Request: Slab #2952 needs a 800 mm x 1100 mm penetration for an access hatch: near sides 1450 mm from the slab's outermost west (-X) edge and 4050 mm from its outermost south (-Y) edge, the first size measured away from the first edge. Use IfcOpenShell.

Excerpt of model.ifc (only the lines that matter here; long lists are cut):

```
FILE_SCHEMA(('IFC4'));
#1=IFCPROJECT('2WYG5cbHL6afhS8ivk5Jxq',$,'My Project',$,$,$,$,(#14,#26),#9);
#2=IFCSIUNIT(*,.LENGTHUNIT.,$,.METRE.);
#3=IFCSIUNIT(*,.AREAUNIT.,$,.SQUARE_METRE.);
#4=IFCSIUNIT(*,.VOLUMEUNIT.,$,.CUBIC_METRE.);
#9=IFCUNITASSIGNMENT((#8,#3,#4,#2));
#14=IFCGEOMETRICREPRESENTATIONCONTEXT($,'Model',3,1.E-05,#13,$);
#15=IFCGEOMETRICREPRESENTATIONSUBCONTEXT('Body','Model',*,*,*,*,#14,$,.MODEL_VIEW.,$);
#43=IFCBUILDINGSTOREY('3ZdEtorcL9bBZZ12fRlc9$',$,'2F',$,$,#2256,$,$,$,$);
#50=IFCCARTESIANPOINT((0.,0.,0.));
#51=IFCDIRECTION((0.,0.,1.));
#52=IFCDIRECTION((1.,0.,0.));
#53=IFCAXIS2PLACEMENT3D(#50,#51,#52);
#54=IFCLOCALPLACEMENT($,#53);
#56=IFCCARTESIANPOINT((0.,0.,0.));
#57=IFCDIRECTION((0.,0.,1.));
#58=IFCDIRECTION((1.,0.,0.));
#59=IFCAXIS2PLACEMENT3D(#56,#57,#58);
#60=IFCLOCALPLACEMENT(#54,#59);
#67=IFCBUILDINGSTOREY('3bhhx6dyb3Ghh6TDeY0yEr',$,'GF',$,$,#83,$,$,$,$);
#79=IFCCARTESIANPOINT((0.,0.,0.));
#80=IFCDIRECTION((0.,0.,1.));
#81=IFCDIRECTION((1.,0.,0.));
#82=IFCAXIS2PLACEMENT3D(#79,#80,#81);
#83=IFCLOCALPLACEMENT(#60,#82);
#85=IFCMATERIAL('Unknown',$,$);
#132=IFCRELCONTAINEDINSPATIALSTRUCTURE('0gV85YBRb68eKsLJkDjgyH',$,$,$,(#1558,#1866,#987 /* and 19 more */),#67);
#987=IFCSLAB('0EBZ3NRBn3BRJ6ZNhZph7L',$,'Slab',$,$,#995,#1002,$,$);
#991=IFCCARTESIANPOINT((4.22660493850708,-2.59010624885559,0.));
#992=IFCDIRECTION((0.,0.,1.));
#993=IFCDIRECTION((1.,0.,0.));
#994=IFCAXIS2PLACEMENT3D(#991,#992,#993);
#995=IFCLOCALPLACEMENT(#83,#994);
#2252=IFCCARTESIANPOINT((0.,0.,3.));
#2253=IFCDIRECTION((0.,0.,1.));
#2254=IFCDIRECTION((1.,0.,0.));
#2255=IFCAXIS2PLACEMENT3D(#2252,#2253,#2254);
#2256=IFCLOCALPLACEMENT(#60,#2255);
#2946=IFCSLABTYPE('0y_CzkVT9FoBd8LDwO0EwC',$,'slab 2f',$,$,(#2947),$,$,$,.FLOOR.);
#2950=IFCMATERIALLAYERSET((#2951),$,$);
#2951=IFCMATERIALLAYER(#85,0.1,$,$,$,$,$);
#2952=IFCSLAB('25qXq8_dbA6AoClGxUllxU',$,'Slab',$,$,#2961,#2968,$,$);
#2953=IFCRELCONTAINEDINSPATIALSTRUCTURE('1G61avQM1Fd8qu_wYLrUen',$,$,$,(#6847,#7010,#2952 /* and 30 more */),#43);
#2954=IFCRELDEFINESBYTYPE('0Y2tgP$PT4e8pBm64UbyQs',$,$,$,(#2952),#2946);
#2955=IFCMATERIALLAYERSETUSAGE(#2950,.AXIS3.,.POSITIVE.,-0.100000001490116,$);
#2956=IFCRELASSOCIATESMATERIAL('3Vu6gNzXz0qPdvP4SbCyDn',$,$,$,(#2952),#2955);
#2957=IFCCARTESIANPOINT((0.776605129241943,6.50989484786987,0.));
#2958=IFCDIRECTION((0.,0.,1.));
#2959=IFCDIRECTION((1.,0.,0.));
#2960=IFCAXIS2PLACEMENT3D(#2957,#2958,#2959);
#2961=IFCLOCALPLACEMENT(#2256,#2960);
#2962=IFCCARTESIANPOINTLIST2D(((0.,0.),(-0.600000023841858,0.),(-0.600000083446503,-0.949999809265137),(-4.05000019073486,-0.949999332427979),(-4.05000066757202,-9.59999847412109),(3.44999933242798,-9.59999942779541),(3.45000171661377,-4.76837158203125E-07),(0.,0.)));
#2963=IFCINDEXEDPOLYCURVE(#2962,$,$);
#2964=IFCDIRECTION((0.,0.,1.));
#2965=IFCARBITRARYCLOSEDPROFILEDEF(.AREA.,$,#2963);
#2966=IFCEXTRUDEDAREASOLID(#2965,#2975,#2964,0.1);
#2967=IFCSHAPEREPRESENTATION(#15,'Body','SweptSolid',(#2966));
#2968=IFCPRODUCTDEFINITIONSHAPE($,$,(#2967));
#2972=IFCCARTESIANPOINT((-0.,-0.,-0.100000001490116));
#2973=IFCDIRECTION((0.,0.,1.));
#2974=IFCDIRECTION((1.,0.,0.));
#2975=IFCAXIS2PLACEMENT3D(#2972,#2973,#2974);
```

```python
import numpy as np
import ifcopenshell
import ifcopenshell.api.feature
import ifcopenshell.api.geometry
import ifcopenshell.api.root
import ifcopenshell.geom
import ifcopenshell.util.placement
import ifcopenshell.util.representation
import ifcopenshell.util.shape
import ifcopenshell.util.unit

model = ifcopenshell.open("model.ifc")
unit_scale = ifcopenshell.util.unit.calculate_unit_scale(model)
settings = ifcopenshell.geom.settings()


def volume(element):
    """Net volume in cubic metres, openings subtracted."""
    shape = ifcopenshell.geom.create_shape(settings, element)
    return ifcopenshell.util.shape.get_volume(shape.geometry)


slab = model.by_guid("25qXq8_dbA6AoClGxUllxU")
before = volume(slab)

# Extent in the slab's own axes, in metres. The edges named are its -X and -Y sides.
slab_shape = ifcopenshell.geom.create_shape(settings, slab)
vertices = ifcopenshell.util.shape.get_vertices(slab_shape.geometry)
x_min, y_min, bottom = vertices.min(axis=0)
top = vertices[:, 2].max()

opening = ifcopenshell.api.root.create_entity(model, ifc_class="IfcOpeningElement", name="Access hatch opening", predefined_type="OPENING")
context = ifcopenshell.util.representation.get_context(model, "Model", "Body", "MODEL_VIEW")
width, depth = 0.8, 1.1
outline = [(0.0, 0.0), (width, 0.0), (width, depth), (0.0, depth), (0.0, 0.0)]
# Overshoot both faces by 50 mm so the cut is clean.
shape = ifcopenshell.api.geometry.add_slab_representation(
    model, context=context, depth=top - bottom + 0.1, polyline=outline
)
ifcopenshell.api.geometry.assign_representation(model, product=opening, representation=shape)

matrix = ifcopenshell.util.placement.get_local_placement(slab.ObjectPlacement)
matrix[:, 3] = matrix @ np.append(np.array([x_min + 1.45, y_min + 4.05, bottom - 0.05]) / unit_scale, 1.0)
ifcopenshell.api.geometry.edit_object_placement(model, product=opening, matrix=matrix, is_si=False)
ifcopenshell.api.feature.add_feature(model, feature=opening, element=slab)

after = volume(slab)

print(f"slab volume {before:.3f} -> {after:.3f} m3")

model.write("model_v2.ifc")
```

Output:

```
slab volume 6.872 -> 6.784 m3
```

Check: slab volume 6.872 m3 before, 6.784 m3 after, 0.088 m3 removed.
